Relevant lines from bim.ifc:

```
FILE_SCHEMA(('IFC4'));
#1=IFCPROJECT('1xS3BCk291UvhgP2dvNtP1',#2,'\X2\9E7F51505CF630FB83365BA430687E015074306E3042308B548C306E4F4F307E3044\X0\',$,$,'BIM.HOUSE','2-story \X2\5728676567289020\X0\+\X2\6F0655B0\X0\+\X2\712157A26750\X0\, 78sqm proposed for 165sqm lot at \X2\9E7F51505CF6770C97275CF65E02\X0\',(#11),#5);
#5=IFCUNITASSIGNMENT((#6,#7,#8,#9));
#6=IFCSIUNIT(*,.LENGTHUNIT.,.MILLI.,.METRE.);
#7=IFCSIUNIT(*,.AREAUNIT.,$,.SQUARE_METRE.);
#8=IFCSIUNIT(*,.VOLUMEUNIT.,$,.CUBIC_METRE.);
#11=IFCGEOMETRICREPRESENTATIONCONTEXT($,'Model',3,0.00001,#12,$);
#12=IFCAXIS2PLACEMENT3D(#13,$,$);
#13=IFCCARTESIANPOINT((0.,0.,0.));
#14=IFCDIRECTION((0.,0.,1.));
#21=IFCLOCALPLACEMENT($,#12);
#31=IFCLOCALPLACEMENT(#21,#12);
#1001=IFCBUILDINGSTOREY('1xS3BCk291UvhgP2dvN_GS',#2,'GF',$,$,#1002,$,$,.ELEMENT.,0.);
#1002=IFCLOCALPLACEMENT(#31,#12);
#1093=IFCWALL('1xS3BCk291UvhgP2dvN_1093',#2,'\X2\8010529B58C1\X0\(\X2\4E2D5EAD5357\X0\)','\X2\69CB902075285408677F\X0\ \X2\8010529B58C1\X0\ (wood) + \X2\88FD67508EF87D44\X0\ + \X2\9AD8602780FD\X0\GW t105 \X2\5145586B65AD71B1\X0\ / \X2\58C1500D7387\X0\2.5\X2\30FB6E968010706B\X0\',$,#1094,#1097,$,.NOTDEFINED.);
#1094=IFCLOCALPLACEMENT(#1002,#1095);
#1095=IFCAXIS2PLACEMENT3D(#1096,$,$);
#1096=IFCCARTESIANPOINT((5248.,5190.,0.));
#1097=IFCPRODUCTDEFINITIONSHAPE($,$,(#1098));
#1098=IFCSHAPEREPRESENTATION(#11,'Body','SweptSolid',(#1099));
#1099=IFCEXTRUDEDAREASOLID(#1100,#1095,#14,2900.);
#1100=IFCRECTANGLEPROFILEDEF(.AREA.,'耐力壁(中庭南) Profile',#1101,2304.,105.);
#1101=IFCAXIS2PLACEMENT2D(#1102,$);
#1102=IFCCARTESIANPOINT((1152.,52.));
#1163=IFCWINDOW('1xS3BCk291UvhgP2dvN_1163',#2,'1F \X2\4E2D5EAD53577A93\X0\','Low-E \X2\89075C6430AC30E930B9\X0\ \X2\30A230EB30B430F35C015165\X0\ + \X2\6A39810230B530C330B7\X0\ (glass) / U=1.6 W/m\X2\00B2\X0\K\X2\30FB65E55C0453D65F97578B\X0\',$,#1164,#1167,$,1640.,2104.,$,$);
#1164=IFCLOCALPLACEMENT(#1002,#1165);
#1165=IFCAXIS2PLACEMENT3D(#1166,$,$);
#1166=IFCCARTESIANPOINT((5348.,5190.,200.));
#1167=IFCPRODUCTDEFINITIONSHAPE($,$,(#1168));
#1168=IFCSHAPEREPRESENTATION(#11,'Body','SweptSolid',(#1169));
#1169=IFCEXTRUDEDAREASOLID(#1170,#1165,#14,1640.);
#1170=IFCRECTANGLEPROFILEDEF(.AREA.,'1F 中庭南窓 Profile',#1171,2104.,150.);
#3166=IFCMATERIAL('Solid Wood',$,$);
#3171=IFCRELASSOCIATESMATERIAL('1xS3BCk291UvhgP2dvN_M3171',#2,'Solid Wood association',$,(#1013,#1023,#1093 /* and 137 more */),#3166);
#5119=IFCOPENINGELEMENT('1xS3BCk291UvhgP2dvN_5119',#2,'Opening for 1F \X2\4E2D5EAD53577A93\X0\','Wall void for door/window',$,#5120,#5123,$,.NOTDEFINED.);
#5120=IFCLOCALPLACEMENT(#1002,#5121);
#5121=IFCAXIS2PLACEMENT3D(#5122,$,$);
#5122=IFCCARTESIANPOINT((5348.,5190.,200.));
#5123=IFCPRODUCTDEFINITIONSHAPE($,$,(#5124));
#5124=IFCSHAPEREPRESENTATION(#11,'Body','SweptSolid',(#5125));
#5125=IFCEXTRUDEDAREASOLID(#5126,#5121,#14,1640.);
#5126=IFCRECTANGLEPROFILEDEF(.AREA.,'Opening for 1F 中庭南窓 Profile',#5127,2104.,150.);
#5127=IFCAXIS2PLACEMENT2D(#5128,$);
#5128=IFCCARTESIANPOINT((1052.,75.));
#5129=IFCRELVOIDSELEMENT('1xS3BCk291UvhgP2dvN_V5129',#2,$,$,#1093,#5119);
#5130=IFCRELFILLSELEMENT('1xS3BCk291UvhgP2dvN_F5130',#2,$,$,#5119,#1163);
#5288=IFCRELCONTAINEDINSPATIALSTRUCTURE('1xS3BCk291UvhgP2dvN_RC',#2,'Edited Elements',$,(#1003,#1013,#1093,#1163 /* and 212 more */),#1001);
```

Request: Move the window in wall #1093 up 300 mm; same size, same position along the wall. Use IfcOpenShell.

```python
import numpy as np
import ifcopenshell
import ifcopenshell.api.geometry
import ifcopenshell.util.placement
import ifcopenshell.util.unit

model = ifcopenshell.open("bim.ifc")
unit_scale = ifcopenshell.util.unit.calculate_unit_scale(model)

window = model.by_guid("1xS3BCk291UvhgP2dvN_1163")
opening = window.FillsVoids[0].RelatingOpeningElement
dz = 300.0

shift = np.array([0.0, 0.0, dz])
# The window is not placed relative to its opening, so move both.
for product in (opening, window):
    matrix = ifcopenshell.util.placement.get_local_placement(product.ObjectPlacement)
    matrix[:3, 3] += shift
    ifcopenshell.api.geometry.edit_object_placement(model, product=product, matrix=matrix, is_si=False)

print(f"moved by {dz * unit_scale:+.3f} m")

model.write("bim_updated.ifc")
```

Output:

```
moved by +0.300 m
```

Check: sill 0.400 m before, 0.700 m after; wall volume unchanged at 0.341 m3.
